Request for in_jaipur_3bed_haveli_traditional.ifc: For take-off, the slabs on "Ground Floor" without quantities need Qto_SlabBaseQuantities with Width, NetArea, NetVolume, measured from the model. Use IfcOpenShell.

First a look at what the model holds.

```python
import ifcopenshell
import ifcopenshell.util.element
import ifcopenshell.util.unit

model = ifcopenshell.open("in_jaipur_3bed_haveli_traditional.ifc")
print(model.schema)
for unit_type in ("LENGTHUNIT", "AREAUNIT", "VOLUMEUNIT"):
    print(unit_type, ifcopenshell.util.unit.calculate_unit_scale(model, unit_type))
storey = next(s for s in model.by_type("IfcBuildingStorey") if s.Name == "Ground Floor")
slabs = [e for e in ifcopenshell.util.element.get_decomposition(storey) if e.is_a("IfcSlab")]
for e in sorted(slabs, key=lambda e: e.id()):
    print(e.id(), e.is_a(), e.Name, list(ifcopenshell.util.element.get_psets(e, qtos_only=True)), sep=" | ")
```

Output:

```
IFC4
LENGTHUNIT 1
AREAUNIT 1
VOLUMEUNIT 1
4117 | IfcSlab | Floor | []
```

```python
import ifcopenshell
import ifcopenshell.api.pset
import ifcopenshell.geom
import ifcopenshell.util.element
import ifcopenshell.util.shape
import ifcopenshell.util.unit

model = ifcopenshell.open("in_jaipur_3bed_haveli_traditional.ifc")
unit_scale = ifcopenshell.util.unit.calculate_unit_scale(model)
area_scale = ifcopenshell.util.unit.calculate_unit_scale(model, "AREAUNIT")
volume_scale = ifcopenshell.util.unit.calculate_unit_scale(model, "VOLUMEUNIT")
settings = ifcopenshell.geom.settings()

storey = next(s for s in model.by_type("IfcBuildingStorey") if s.Name == "Ground Floor")
slabs = [e for e in ifcopenshell.util.element.get_decomposition(storey) if e.is_a("IfcSlab")]

for e in sorted(slabs, key=lambda e: e.id()):
    if ifcopenshell.util.element.get_psets(e, qtos_only=True, should_inherit=False):
        continue
    # Geometry comes back in metres, in the element's own axes.
    shape = ifcopenshell.geom.create_shape(settings, e)
    values = {
        "Width": ifcopenshell.util.shape.get_z(shape.geometry) / unit_scale,
        "NetArea": ifcopenshell.util.shape.get_footprint_area(shape.geometry) / area_scale,
        "NetVolume": ifcopenshell.util.shape.get_volume(shape.geometry) / volume_scale,
    }
    qto = ifcopenshell.api.pset.add_qto(model, product=e, name="Qto_SlabBaseQuantities")
    ifcopenshell.api.pset.edit_qto(model, qto=qto, properties=values)
    print(e.id(), {k: round(v, 3) for k, v in values.items()})

model.write("in_jaipur_3bed_haveli_traditional_v2.ifc")
```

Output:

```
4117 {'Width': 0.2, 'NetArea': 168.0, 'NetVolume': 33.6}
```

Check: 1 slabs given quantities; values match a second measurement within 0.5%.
